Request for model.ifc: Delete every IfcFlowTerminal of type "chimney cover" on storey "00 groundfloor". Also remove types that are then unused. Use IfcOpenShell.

First a look at what the model holds.

```python
import ifcopenshell
import ifcopenshell.util.element

model = ifcopenshell.open("model.ifc")
print(model.schema)
storey = next(s for s in model.by_type("IfcBuildingStorey") if s.Name == "00 groundfloor")
terminals = [e for e in ifcopenshell.util.element.get_decomposition(storey) if e.is_a("IfcFlowTerminal")]
seen = {}
for e in terminals:
    element_type = ifcopenshell.util.element.get_type(e)
    name = element_type.Name if element_type not in (None, e) else None
    seen[name] = seen.get(name, 0) + 1
for name, count in sorted(seen.items(), key=str):
    print(count, "x", name)
```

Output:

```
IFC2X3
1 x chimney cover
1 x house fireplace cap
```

```python
import ifcopenshell
import ifcopenshell.api.root
import ifcopenshell.util.element

model = ifcopenshell.open("model.ifc")

storey = next(s for s in model.by_type("IfcBuildingStorey") if s.Name == "00 groundfloor")
terminals = [e for e in ifcopenshell.util.element.get_decomposition(storey) if e.is_a("IfcFlowTerminal")]
targets = [e for e in terminals if (t := ifcopenshell.util.element.get_type(e)) not in (None, e) and t.Name == "chimney cover"]
types = {ifcopenshell.util.element.get_type(e) for e in targets} - {None, *targets}

for e in targets:
    ifcopenshell.api.root.remove_product(model, product=e)
print(len(targets), "removed")

unused = [t for t in types if not ifcopenshell.util.element.get_types(t)]
for t in unused:
    ifcopenshell.api.root.remove_product(model, product=t)
print(len(unused), "unused types removed")

model.write("model_updated.ifc")
```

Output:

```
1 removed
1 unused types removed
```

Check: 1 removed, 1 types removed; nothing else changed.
